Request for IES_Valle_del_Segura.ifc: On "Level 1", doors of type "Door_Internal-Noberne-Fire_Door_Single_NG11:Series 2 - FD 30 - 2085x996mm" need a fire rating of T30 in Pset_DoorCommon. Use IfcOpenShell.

First a look at what the model holds.

```python
import ifcopenshell
import ifcopenshell.util.element

model = ifcopenshell.open("IES_Valle_del_Segura.ifc")
print(model.schema)
storey = next(s for s in model.by_type("IfcBuildingStorey") if s.Name == "Level 1")
doors = [e for e in ifcopenshell.util.element.get_decomposition(storey) if e.is_a("IfcDoor")]
seen = {}
for e in doors:
    element_type = ifcopenshell.util.element.get_type(e)
    key = (element_type.Name if element_type != e and element_type else None, ifcopenshell.util.element.get_pset(e, "Pset_DoorCommon", "FireRating"))
    seen[key] = seen.get(key, 0) + 1
for (name, value), count in sorted(seen.items(), key=str):
    print(count, "x", name, "|", value)
```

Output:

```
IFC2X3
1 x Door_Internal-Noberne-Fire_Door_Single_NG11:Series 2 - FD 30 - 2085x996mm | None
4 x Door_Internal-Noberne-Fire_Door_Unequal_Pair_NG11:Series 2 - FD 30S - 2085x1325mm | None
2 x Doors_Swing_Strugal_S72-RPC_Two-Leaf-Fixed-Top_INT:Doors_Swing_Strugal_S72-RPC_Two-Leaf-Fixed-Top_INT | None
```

```python
import ifcopenshell
import ifcopenshell.api.pset
import ifcopenshell.util.element

model = ifcopenshell.open("IES_Valle_del_Segura.ifc")

storey = next(s for s in model.by_type("IfcBuildingStorey") if s.Name == "Level 1")
doors = [e for e in ifcopenshell.util.element.get_decomposition(storey) if e.is_a("IfcDoor")]

count = 0
for e in doors:
    element_type = ifcopenshell.util.element.get_type(e)
    if element_type in (None, e) or element_type.Name != "Door_Internal-Noberne-Fire_Door_Single_NG11:Series 2 - FD 30 - 2085x996mm":
        continue
    # add_pset returns the element's existing set when there is one.
    pset = ifcopenshell.api.pset.add_pset(model, product=e, name="Pset_DoorCommon")
    ifcopenshell.api.pset.edit_pset(model, pset=pset, properties={"FireRating": "T30"})
    count += 1

print(count, "doors updated")

model.write("IES_Valle_del_Segura_updated.ifc")
```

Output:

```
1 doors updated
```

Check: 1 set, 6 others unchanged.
